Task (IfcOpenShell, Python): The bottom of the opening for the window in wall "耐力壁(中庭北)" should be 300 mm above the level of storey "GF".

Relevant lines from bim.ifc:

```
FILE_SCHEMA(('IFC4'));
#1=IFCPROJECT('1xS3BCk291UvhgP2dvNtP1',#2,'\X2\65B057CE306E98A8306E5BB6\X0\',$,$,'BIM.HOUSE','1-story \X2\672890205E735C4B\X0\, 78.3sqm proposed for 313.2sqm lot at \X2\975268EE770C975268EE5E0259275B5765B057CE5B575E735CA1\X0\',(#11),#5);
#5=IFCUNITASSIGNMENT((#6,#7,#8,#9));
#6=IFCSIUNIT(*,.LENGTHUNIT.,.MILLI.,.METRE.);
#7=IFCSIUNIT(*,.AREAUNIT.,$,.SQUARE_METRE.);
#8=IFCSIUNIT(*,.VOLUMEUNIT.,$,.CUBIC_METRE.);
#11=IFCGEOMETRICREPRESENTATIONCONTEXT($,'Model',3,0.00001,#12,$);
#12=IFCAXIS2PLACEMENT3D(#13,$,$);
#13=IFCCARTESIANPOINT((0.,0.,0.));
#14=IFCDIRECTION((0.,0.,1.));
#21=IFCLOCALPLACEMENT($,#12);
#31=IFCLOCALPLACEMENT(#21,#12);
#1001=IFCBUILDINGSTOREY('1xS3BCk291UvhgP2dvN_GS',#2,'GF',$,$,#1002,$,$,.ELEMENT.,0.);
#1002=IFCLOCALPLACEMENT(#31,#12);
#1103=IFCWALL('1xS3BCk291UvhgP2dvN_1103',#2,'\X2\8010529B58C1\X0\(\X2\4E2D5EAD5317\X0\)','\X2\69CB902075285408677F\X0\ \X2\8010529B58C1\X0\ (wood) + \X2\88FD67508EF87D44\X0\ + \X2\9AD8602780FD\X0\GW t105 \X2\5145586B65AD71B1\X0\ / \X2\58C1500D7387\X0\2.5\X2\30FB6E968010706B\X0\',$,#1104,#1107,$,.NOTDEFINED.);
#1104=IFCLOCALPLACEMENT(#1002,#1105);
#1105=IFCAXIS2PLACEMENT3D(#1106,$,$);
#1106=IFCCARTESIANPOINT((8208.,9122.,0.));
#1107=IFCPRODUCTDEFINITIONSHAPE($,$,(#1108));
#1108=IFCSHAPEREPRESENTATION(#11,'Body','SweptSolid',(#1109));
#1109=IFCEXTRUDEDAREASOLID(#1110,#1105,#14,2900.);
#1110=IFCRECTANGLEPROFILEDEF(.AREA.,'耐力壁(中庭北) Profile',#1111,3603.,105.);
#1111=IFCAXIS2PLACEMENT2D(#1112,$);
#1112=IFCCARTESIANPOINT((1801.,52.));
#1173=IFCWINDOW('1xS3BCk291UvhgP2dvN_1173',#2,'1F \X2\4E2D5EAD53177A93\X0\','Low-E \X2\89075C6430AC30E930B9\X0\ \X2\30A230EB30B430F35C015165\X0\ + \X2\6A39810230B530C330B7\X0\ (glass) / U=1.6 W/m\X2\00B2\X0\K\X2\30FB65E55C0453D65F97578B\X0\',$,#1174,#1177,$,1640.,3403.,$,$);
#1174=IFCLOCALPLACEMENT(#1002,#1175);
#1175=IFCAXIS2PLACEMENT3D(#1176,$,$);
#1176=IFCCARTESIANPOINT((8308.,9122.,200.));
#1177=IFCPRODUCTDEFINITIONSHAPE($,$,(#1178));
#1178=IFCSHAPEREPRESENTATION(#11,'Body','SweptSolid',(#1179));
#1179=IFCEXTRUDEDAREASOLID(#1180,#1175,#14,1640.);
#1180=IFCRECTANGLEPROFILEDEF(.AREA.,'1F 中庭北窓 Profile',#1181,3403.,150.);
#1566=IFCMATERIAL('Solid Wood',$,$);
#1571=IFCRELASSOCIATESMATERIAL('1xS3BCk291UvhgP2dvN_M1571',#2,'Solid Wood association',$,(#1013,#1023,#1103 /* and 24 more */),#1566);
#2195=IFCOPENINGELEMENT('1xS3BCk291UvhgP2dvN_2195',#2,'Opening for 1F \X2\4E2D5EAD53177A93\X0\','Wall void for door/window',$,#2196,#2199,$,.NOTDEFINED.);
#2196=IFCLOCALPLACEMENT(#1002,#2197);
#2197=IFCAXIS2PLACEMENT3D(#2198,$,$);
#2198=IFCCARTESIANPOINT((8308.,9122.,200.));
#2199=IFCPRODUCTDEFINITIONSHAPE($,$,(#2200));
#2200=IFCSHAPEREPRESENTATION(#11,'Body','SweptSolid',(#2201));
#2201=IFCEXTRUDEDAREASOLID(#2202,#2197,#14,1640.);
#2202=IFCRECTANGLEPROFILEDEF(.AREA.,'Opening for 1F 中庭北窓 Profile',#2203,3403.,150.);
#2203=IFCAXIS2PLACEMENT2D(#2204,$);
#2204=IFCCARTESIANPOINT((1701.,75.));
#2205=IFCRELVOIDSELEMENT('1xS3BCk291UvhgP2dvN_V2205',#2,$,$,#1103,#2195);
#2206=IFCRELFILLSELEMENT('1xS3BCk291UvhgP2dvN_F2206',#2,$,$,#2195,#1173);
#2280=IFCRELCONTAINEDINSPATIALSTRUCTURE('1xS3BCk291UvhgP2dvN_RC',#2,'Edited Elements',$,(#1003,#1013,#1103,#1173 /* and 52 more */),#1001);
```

```python
import numpy as np
import ifcopenshell
import ifcopenshell.api.geometry
import ifcopenshell.geom
import ifcopenshell.util.element
import ifcopenshell.util.placement
import ifcopenshell.util.shape
import ifcopenshell.util.unit

model = ifcopenshell.open("bim.ifc")
unit_scale = ifcopenshell.util.unit.calculate_unit_scale(model)

window = model.by_guid("1xS3BCk291UvhgP2dvN_1173")
opening = window.FillsVoids[0].RelatingOpeningElement
storey = ifcopenshell.util.element.get_container(window, ifc_class="IfcBuildingStorey")
level = ifcopenshell.util.placement.get_local_placement(storey.ObjectPlacement)[2, 3]

# The opening's origin need not be at the sill, so measure its lowest point.
shape = ifcopenshell.geom.create_shape(ifcopenshell.geom.settings(), opening)
bottom = ifcopenshell.util.shape.get_shape_bottom_elevation(shape, shape.geometry) / unit_scale
dz = level + 300.0 - bottom

shift = np.array([0.0, 0.0, dz])
# The window is not placed relative to its opening, so move both.
for product in (opening, window):
    matrix = ifcopenshell.util.placement.get_local_placement(product.ObjectPlacement)
    matrix[:3, 3] += shift
    ifcopenshell.api.geometry.edit_object_placement(model, product=product, matrix=matrix, is_si=False)

print(f"moved by {dz * unit_scale:+.3f} m")

model.write("bim_edited.ifc")
```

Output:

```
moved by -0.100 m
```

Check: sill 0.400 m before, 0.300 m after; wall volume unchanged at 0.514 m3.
